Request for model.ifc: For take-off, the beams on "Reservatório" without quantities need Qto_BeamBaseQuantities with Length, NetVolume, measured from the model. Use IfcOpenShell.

First a look at what the model holds.

```python
import ifcopenshell
import ifcopenshell.util.element
import ifcopenshell.util.unit

model = ifcopenshell.open("model.ifc")
print(model.schema)
for unit_type in ("LENGTHUNIT", "AREAUNIT", "VOLUMEUNIT"):
    print(unit_type, ifcopenshell.util.unit.calculate_unit_scale(model, unit_type))
storey = next(s for s in model.by_type("IfcBuildingStorey") if s.Name == "Reservatório")
beams = [e for e in ifcopenshell.util.element.get_decomposition(storey) if e.is_a("IfcBeam")]
for e in sorted(beams, key=lambda e: e.id()):
    print(e.id(), e.is_a(), e.Name, list(ifcopenshell.util.element.get_psets(e, qtos_only=True)), sep=" | ")
```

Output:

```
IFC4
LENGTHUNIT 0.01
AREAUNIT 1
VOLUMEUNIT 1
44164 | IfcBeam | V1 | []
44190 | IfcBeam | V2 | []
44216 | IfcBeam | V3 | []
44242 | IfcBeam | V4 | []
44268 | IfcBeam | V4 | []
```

```python
import ifcopenshell
import ifcopenshell.api.pset
import ifcopenshell.geom
import ifcopenshell.util.element
import ifcopenshell.util.shape
import ifcopenshell.util.unit

model = ifcopenshell.open("model.ifc")
unit_scale = ifcopenshell.util.unit.calculate_unit_scale(model)
volume_scale = ifcopenshell.util.unit.calculate_unit_scale(model, "VOLUMEUNIT")
settings = ifcopenshell.geom.settings()

storey = next(s for s in model.by_type("IfcBuildingStorey") if s.Name == "Reservatório")
beams = [e for e in ifcopenshell.util.element.get_decomposition(storey) if e.is_a("IfcBeam")]

for e in sorted(beams, key=lambda e: e.id()):
    if ifcopenshell.util.element.get_psets(e, qtos_only=True, should_inherit=False):
        continue
    # Geometry comes back in metres, in the element's own axes.
    shape = ifcopenshell.geom.create_shape(settings, e)
    values = {
        "Length": ifcopenshell.util.shape.get_max_xyz(shape.geometry) / unit_scale,
        "NetVolume": ifcopenshell.util.shape.get_volume(shape.geometry) / volume_scale,
    }
    qto = ifcopenshell.api.pset.add_qto(model, product=e, name="Qto_BeamBaseQuantities")
    ifcopenshell.api.pset.edit_qto(model, qto=qto, properties=values)
    print(e.id(), {k: round(v, 3) for k, v in values.items()})

model.write("model_edited.ifc")
```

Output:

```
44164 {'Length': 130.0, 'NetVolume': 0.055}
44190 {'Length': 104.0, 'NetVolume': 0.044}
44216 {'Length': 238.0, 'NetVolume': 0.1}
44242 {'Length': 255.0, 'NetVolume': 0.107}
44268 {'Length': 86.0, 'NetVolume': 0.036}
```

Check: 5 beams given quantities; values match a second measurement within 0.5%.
